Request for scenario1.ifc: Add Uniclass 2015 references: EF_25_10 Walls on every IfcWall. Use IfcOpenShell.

First a look at what the model holds.

```python
import ifcopenshell

model = ifcopenshell.open("scenario1.ifc")
print(model.schema)
print("classifications:", [c.Name for c in model.by_type("IfcClassification")])
for ifc_class in ("IfcDoor", "IfcRoof", "IfcStair", "IfcWall", "IfcWindow"):
    print(ifc_class, len(model.by_type(ifc_class)))
```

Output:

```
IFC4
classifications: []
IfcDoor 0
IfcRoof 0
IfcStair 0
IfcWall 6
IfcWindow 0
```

```python
import ifcopenshell
import ifcopenshell.api.classification

model = ifcopenshell.open("scenario1.ifc")

system = ifcopenshell.api.classification.add_classification(model, classification="Uniclass 2015")

codes = {
    "IfcWall": ("EF_25_10", "Walls"),
}
for ifc_class, (code, name) in codes.items():
    products = model.by_type(ifc_class)
    ifcopenshell.api.classification.add_reference(
        model, products=products, classification=system, identification=code, name=name
    )
    print(code, len(products))

model.write("scenario1-out.ifc")
```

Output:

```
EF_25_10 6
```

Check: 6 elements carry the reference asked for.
